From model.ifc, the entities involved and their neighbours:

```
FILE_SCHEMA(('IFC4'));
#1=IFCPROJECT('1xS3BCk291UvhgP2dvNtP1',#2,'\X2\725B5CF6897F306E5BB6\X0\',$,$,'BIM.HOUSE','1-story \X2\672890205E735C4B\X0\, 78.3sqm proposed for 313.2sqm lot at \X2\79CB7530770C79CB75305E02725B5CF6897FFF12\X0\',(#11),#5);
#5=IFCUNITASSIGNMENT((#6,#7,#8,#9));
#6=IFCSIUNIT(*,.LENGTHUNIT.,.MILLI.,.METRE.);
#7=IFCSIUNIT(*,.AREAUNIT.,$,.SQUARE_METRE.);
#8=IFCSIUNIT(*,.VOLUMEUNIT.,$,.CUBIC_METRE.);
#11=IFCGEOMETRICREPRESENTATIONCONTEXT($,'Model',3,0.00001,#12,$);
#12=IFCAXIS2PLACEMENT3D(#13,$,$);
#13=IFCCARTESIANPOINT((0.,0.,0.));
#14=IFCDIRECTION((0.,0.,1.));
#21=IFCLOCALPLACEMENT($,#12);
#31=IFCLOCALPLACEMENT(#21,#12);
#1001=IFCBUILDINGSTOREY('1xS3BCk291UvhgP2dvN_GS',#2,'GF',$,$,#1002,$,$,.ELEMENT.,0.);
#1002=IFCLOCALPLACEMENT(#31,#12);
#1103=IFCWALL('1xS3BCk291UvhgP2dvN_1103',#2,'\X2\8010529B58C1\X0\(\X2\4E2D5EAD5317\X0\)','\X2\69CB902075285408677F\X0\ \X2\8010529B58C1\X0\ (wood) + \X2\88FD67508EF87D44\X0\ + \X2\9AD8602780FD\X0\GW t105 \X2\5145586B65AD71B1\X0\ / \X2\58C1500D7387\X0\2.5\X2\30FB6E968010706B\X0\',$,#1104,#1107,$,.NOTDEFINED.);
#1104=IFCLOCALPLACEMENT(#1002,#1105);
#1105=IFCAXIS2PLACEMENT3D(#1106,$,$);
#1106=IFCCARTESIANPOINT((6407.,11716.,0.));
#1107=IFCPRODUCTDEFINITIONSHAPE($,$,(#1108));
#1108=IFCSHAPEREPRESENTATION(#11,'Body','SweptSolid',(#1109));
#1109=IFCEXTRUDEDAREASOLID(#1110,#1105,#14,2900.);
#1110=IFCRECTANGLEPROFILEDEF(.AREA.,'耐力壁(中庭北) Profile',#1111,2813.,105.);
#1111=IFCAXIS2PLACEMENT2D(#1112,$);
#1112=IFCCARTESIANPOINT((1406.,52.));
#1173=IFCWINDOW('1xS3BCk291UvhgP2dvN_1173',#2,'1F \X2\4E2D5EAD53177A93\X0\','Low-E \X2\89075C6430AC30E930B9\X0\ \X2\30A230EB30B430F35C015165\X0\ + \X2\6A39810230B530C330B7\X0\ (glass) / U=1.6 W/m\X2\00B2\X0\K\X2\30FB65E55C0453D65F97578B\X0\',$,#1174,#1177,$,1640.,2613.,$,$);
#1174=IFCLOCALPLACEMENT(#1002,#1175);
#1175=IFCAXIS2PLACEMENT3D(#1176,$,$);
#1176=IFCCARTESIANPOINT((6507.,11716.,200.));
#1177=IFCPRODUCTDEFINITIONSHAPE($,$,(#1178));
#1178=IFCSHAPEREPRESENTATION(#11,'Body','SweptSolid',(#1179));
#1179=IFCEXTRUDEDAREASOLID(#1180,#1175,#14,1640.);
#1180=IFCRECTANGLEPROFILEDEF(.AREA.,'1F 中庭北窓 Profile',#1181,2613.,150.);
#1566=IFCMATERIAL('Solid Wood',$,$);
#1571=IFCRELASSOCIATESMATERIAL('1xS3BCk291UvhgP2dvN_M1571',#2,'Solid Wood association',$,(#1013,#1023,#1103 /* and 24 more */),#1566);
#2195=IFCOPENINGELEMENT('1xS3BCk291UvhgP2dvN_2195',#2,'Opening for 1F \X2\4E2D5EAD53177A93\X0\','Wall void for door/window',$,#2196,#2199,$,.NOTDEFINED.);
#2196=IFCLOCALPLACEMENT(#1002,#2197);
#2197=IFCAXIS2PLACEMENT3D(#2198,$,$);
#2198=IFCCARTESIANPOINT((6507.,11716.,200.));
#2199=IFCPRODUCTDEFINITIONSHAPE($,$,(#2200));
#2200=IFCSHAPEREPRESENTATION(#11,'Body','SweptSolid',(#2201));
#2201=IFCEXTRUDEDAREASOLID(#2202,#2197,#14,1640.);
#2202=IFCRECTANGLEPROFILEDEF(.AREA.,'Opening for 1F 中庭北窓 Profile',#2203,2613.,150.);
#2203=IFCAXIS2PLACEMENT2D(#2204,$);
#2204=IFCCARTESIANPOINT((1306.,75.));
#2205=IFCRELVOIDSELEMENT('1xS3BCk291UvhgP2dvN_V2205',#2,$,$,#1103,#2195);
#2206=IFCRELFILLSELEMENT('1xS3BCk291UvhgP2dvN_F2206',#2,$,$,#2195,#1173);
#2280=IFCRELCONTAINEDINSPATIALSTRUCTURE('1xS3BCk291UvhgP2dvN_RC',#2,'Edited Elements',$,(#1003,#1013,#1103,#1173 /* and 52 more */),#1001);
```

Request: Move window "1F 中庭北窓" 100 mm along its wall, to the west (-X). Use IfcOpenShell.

```python
import ifcopenshell
import ifcopenshell.api.geometry
import ifcopenshell.util.placement
import ifcopenshell.util.unit

model = ifcopenshell.open("model.ifc")
unit_scale = ifcopenshell.util.unit.calculate_unit_scale(model)

window = model.by_guid("1xS3BCk291UvhgP2dvN_1173")
opening = window.FillsVoids[0].RelatingOpeningElement
wall = opening.VoidsElements[0].RelatingBuildingElement

wall_matrix = ifcopenshell.util.placement.get_local_placement(wall.ObjectPlacement)
shift = wall_matrix[:3, 0] * -0.1 / unit_scale
before = ifcopenshell.util.placement.get_local_placement(window.ObjectPlacement)[:3, 3].copy()

# The window is not placed relative to its opening, so move both.
for product in (opening, window):
    matrix = ifcopenshell.util.placement.get_local_placement(product.ObjectPlacement)
    matrix[:3, 3] += shift
    ifcopenshell.api.geometry.edit_object_placement(model, product=product, matrix=matrix, is_si=False)

after = ifcopenshell.util.placement.get_local_placement(window.ObjectPlacement)[:3, 3]
print("window moved by", (after - before).round(3) + 0.0)

model.write("model_rev.ifc")
```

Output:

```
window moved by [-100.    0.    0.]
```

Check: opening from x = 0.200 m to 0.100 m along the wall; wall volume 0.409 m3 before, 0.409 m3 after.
